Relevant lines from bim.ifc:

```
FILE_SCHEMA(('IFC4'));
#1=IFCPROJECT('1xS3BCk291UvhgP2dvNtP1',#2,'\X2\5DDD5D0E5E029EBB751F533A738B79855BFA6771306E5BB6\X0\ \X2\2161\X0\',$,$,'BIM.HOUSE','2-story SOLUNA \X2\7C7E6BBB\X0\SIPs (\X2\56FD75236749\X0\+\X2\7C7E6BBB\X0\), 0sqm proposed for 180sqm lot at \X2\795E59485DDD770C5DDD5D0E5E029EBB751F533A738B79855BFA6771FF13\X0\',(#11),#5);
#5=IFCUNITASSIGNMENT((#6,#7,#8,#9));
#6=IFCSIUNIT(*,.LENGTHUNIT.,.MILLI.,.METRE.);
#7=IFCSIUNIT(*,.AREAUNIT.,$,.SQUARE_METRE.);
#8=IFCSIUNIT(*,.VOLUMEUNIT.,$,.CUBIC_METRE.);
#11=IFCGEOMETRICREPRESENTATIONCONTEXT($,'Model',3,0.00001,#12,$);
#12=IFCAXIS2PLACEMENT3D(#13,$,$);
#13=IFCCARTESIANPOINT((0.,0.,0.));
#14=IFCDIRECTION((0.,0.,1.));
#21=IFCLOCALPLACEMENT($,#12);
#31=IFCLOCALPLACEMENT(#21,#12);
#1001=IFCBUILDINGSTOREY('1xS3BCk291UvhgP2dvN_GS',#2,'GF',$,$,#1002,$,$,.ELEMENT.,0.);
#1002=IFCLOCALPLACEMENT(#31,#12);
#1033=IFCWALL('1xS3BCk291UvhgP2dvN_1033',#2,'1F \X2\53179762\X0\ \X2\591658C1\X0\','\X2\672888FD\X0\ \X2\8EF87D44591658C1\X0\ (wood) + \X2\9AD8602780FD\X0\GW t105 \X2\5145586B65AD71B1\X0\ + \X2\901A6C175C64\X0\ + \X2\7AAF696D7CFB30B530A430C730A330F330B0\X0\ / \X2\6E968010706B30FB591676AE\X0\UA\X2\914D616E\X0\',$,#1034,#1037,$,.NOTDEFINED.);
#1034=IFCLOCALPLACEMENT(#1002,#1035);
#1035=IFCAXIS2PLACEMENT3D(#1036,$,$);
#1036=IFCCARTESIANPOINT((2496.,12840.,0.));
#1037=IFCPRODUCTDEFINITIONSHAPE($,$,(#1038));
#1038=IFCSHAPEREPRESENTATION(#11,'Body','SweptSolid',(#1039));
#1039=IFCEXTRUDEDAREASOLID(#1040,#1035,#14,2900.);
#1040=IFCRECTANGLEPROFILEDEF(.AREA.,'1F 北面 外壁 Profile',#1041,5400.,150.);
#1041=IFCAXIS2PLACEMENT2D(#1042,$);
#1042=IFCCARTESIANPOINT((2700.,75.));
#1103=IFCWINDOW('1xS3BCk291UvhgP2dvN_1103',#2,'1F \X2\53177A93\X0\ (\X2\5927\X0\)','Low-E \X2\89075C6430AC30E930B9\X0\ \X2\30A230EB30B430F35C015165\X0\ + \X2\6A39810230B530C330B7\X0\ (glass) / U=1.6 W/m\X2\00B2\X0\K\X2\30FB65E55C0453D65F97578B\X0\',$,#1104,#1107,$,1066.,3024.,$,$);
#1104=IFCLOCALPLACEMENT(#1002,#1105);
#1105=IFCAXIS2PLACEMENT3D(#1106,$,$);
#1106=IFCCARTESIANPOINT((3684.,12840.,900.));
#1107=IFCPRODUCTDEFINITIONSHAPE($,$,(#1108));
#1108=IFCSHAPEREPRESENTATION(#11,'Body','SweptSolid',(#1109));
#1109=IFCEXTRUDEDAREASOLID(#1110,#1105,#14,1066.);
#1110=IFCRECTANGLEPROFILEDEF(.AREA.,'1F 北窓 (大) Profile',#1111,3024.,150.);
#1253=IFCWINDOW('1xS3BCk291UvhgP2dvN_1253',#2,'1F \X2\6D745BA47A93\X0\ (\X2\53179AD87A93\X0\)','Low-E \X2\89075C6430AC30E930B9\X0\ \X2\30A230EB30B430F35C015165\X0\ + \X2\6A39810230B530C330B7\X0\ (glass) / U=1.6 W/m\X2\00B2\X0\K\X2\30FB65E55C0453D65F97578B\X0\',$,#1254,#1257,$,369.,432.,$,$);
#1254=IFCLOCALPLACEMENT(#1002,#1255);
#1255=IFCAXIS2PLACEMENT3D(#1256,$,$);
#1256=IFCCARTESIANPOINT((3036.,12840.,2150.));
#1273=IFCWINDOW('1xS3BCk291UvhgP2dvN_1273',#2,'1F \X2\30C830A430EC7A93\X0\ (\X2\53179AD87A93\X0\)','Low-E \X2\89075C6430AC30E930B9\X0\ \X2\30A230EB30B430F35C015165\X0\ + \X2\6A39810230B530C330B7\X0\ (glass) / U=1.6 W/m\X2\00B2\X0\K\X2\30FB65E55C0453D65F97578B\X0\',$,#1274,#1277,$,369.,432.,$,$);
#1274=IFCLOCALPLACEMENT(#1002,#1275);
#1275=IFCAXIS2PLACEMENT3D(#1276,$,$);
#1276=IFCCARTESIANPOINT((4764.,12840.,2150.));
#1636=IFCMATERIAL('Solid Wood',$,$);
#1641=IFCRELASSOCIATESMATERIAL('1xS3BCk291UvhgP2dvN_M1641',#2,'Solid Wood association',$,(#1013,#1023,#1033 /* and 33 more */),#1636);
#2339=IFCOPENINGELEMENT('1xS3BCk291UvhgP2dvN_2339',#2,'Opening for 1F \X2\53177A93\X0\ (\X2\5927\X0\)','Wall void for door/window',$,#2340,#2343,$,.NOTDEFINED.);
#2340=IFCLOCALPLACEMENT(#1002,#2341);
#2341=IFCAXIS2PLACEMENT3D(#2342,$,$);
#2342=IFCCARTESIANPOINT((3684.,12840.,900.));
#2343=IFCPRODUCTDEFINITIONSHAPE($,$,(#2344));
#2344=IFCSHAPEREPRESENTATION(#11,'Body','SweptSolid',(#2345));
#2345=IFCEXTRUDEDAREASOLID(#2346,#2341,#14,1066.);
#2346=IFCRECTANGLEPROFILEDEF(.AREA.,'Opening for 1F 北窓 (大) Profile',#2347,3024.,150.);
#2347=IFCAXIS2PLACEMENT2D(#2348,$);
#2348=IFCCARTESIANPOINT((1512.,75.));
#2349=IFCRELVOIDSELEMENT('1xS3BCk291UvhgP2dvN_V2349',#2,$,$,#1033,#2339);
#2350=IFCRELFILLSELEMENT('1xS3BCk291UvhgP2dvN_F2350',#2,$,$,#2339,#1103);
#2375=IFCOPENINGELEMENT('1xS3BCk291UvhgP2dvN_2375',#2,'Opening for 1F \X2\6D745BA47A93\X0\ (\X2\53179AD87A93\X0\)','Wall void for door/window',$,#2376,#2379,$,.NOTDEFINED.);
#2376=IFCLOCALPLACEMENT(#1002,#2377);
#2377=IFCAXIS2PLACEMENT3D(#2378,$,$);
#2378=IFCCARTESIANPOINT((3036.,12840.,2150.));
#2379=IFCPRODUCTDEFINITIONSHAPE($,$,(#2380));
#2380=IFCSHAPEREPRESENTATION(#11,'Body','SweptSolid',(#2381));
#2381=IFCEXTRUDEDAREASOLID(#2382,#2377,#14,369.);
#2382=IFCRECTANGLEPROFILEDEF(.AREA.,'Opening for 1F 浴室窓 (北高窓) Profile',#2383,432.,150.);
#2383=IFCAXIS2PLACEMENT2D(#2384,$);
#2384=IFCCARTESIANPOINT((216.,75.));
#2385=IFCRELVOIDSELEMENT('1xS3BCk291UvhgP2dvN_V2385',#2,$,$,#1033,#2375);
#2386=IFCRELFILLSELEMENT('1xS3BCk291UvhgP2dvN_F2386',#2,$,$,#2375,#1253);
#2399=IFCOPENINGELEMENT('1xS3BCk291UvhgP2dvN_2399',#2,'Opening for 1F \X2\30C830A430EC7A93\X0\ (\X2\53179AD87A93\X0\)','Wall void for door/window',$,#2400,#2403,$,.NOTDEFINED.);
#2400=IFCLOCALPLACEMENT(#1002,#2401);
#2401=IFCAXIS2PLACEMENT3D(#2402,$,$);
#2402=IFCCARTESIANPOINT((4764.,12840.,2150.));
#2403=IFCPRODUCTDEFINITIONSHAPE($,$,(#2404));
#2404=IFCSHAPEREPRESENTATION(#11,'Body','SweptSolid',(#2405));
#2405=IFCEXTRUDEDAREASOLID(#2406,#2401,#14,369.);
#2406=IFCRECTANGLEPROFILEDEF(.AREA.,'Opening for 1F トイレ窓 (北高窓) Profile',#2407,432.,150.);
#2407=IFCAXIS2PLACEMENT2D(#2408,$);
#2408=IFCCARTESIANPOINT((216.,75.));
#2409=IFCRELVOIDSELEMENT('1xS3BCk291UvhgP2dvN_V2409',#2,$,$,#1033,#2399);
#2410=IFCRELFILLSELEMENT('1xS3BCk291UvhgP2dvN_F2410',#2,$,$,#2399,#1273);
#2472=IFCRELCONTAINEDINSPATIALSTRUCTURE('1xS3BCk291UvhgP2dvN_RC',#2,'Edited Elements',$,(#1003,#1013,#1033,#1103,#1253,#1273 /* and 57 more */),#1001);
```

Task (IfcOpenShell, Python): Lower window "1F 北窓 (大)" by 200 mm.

```python
import numpy as np
import ifcopenshell
import ifcopenshell.api.geometry
import ifcopenshell.util.placement
import ifcopenshell.util.unit

model = ifcopenshell.open("bim.ifc")
unit_scale = ifcopenshell.util.unit.calculate_unit_scale(model)

window = model.by_guid("1xS3BCk291UvhgP2dvN_1103")
opening = window.FillsVoids[0].RelatingOpeningElement
dz = -0.2 / unit_scale

shift = np.array([0.0, 0.0, dz])
# The window is not placed relative to its opening, so move both.
for product in (opening, window):
    matrix = ifcopenshell.util.placement.get_local_placement(product.ObjectPlacement)
    matrix[:3, 3] += shift
    ifcopenshell.api.geometry.edit_object_placement(model, product=product, matrix=matrix, is_si=False)

print(f"moved by {dz * unit_scale:+.3f} m")

model.write("bim_v2.ifc")
```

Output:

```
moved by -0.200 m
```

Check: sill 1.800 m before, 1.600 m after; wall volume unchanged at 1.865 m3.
